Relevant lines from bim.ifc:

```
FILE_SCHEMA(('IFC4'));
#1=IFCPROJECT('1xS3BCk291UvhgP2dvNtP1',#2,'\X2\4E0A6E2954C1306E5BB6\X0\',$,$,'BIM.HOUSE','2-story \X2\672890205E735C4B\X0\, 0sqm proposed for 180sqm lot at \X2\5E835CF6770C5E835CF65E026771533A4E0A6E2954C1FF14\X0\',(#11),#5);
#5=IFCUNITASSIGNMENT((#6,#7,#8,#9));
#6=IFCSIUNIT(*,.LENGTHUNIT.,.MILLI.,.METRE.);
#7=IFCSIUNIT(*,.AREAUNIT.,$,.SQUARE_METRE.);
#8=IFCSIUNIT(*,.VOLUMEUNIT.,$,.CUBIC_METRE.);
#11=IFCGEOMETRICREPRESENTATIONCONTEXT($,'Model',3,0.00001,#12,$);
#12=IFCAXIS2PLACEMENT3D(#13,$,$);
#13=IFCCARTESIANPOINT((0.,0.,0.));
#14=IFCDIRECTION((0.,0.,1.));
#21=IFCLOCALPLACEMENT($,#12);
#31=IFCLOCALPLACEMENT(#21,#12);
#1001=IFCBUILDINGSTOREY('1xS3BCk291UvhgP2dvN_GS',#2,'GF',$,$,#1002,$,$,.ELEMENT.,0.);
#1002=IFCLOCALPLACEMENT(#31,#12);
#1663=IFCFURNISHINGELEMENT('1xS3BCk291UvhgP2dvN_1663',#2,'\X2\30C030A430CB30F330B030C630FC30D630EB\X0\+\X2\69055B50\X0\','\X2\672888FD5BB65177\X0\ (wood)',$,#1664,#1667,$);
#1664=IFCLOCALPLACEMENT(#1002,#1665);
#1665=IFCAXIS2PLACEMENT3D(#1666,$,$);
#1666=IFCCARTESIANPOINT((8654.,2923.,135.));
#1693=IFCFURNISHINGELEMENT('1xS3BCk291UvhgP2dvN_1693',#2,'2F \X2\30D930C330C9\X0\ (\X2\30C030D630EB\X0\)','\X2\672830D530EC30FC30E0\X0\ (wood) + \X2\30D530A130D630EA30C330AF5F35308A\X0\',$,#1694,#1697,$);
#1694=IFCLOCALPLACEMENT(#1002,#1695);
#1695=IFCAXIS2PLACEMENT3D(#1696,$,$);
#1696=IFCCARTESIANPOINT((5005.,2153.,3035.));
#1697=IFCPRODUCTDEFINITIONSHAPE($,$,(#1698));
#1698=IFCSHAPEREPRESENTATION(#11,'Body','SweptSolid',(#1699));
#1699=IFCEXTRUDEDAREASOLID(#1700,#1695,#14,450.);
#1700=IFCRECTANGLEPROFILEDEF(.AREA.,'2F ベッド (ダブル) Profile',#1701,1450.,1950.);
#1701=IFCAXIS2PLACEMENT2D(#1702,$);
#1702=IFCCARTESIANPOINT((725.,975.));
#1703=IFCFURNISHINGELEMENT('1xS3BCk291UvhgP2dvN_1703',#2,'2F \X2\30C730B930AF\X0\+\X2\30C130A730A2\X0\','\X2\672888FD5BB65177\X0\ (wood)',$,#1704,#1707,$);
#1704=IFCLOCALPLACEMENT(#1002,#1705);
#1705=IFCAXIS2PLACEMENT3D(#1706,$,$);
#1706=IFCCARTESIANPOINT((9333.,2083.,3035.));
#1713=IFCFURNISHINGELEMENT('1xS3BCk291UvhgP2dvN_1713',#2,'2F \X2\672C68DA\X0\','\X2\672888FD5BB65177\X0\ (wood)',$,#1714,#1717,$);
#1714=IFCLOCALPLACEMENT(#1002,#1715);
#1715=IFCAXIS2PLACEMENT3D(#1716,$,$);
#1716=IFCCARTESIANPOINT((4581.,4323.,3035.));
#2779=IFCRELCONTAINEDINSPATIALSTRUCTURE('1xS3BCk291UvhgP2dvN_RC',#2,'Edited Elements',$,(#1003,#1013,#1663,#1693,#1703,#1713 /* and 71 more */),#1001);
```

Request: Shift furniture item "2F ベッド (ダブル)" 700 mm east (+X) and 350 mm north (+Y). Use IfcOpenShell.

```python
import ifcopenshell
import ifcopenshell.api.geometry
import ifcopenshell.util.placement
import ifcopenshell.util.unit

model = ifcopenshell.open("bim.ifc")
unit_scale = ifcopenshell.util.unit.calculate_unit_scale(model)

item = model.by_id(1693)
matrix = ifcopenshell.util.placement.get_local_placement(item.ObjectPlacement)
matrix[0, 3] += 0.7 / unit_scale
matrix[1, 3] += 0.35 / unit_scale
ifcopenshell.api.geometry.edit_object_placement(model, product=item, matrix=matrix, is_si=False)

print(ifcopenshell.util.placement.get_local_placement(item.ObjectPlacement).round(3) + 0.0)

model.write("bim_v2.ifc")
```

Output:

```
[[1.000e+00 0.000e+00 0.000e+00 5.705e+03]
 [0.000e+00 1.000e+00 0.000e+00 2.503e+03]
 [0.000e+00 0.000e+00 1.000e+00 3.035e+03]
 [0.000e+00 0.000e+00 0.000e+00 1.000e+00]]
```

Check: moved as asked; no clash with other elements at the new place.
